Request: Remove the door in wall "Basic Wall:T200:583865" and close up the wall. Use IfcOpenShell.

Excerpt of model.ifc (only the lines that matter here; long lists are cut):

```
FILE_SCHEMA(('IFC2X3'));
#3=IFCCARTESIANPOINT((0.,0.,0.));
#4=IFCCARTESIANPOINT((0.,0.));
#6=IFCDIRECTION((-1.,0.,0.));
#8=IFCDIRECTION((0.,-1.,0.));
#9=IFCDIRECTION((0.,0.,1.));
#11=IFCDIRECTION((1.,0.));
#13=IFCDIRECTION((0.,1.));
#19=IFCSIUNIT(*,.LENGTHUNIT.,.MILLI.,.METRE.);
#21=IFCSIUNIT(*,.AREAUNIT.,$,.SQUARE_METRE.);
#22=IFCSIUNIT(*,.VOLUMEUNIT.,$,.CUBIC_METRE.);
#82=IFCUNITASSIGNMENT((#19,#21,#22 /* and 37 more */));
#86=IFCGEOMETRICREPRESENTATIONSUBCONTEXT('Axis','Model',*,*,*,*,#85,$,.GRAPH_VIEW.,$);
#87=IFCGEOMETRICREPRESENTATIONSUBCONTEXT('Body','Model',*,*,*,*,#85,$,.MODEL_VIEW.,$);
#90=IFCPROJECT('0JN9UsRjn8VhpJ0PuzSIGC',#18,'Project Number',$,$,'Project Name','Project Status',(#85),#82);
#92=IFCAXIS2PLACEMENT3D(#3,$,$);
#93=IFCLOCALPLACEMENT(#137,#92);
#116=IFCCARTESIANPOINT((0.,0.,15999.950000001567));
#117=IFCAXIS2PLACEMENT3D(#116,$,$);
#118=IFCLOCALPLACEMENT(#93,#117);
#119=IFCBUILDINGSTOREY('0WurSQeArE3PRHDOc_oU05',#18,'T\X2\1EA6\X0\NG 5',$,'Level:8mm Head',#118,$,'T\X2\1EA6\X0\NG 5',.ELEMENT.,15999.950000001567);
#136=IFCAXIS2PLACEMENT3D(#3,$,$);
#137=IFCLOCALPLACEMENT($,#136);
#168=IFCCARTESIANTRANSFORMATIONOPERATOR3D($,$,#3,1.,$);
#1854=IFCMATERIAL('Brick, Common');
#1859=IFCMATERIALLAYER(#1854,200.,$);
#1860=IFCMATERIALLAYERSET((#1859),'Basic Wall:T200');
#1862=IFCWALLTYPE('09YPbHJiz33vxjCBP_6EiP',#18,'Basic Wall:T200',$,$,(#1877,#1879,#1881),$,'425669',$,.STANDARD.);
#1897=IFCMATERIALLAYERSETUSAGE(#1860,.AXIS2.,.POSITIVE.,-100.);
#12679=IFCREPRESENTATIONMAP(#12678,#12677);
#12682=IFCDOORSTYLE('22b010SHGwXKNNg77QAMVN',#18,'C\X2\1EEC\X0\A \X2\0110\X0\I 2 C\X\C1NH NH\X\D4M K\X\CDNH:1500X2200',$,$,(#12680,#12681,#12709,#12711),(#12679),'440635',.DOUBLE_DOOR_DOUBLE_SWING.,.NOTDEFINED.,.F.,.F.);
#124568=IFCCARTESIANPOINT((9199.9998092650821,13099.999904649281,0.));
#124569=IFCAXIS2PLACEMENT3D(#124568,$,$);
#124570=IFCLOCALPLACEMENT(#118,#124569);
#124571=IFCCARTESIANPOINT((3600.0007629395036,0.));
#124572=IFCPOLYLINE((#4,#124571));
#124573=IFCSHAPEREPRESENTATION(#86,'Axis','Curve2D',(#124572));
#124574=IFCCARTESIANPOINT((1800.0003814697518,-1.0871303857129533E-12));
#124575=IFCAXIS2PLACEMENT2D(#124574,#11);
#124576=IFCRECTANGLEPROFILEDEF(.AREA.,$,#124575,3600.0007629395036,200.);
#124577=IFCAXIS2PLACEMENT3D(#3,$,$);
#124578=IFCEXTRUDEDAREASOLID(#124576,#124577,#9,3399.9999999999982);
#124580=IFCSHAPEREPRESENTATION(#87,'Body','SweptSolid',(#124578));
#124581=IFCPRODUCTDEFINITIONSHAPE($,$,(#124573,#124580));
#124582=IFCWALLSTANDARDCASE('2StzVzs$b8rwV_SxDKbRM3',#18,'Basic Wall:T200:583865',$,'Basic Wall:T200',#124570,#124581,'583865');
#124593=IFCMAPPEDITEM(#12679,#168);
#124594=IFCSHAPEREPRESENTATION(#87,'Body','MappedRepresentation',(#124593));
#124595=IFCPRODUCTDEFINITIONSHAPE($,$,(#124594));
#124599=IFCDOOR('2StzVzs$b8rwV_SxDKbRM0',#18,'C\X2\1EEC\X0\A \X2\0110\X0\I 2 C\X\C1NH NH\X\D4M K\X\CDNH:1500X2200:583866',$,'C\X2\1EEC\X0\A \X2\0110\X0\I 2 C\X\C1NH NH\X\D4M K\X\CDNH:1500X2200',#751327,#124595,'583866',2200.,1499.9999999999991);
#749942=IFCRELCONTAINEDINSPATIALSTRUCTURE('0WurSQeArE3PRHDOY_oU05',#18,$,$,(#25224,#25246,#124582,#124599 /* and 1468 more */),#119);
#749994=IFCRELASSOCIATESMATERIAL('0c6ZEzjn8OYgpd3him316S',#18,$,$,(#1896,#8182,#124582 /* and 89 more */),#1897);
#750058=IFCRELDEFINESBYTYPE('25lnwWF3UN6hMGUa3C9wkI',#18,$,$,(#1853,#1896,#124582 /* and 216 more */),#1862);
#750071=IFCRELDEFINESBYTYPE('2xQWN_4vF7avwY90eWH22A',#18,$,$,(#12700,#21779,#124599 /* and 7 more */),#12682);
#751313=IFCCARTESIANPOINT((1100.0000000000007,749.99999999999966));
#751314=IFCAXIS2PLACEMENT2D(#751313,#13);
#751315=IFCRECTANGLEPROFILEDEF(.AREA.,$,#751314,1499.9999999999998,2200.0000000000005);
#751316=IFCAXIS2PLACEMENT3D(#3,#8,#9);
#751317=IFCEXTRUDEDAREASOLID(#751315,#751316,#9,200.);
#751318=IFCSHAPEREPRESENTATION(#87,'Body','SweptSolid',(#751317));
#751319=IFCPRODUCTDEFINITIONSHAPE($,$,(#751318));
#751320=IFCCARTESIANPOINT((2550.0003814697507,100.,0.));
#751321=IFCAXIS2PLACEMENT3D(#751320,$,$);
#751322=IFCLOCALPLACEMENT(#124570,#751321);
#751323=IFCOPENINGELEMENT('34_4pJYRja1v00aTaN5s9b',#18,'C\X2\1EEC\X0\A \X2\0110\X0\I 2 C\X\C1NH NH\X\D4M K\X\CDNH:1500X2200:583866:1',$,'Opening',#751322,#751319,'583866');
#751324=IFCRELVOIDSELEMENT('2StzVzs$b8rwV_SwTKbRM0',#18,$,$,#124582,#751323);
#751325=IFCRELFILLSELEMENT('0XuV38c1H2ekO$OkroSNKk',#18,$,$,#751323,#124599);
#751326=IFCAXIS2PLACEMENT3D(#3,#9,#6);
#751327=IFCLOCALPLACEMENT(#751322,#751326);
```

```python
import ifcopenshell
import ifcopenshell.api.feature
import ifcopenshell.api.root
import ifcopenshell.geom
import ifcopenshell.util.shape

model = ifcopenshell.open("model.ifc")
settings = ifcopenshell.geom.settings()


def volume(element):
    """Net volume in cubic metres, openings subtracted."""
    shape = ifcopenshell.geom.create_shape(settings, element)
    return ifcopenshell.util.shape.get_volume(shape.geometry)


door = model.by_guid("2StzVzs$b8rwV_SxDKbRM0")
opening = door.FillsVoids[0].RelatingOpeningElement
wall = opening.VoidsElements[0].RelatingBuildingElement
before = volume(wall)

ifcopenshell.api.root.remove_product(model, product=door)
ifcopenshell.api.feature.remove_feature(model, feature=opening)

after = volume(wall)

print(f"wall volume {before:.3f} -> {after:.3f} m3")

model.write("model_edited.ifc")
```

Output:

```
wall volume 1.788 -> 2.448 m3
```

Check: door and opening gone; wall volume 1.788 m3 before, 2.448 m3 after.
